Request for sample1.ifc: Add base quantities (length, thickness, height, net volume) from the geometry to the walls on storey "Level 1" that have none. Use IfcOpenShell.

First a look at what the model holds.

```python
import ifcopenshell
import ifcopenshell.util.element
import ifcopenshell.util.unit

model = ifcopenshell.open("sample1.ifc")
print(model.schema)
for unit_type in ("LENGTHUNIT", "AREAUNIT", "VOLUMEUNIT"):
    print(unit_type, ifcopenshell.util.unit.calculate_unit_scale(model, unit_type))
storey = next(s for s in model.by_type("IfcBuildingStorey") if s.Name == "Level 1")
walls = [e for e in ifcopenshell.util.element.get_decomposition(storey) if e.is_a("IfcWall")]
for e in sorted(walls, key=lambda e: e.id()):
    print(e.id(), e.is_a(), e.Name, list(ifcopenshell.util.element.get_psets(e, qtos_only=True)), sep=" | ")
```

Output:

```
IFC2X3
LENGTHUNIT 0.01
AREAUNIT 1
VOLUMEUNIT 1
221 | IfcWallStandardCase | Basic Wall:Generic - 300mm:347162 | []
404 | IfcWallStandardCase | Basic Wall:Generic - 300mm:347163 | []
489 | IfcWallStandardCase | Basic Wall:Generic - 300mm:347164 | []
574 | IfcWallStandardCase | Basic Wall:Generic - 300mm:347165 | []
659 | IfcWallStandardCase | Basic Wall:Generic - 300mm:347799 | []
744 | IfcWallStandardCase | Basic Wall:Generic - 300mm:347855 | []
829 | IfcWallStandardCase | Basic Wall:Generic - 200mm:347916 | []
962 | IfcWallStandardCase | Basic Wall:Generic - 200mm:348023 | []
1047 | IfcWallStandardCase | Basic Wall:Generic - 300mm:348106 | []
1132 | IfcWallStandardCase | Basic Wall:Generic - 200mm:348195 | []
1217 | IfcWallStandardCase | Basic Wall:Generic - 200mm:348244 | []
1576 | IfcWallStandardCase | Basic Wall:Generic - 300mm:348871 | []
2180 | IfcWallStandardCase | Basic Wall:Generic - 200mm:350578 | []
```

```python
import ifcopenshell
import ifcopenshell.api.pset
import ifcopenshell.geom
import ifcopenshell.util.element
import ifcopenshell.util.shape
import ifcopenshell.util.unit

model = ifcopenshell.open("sample1.ifc")
unit_scale = ifcopenshell.util.unit.calculate_unit_scale(model)
volume_scale = ifcopenshell.util.unit.calculate_unit_scale(model, "VOLUMEUNIT")
settings = ifcopenshell.geom.settings()

storey = next(s for s in model.by_type("IfcBuildingStorey") if s.Name == "Level 1")
walls = [e for e in ifcopenshell.util.element.get_decomposition(storey) if e.is_a("IfcWall")]

for e in sorted(walls, key=lambda e: e.id()):
    if ifcopenshell.util.element.get_psets(e, qtos_only=True, should_inherit=False):
        continue
    # Geometry comes back in metres, in the element's own axes.
    shape = ifcopenshell.geom.create_shape(settings, e)
    values = {
        "Length": ifcopenshell.util.shape.get_x(shape.geometry) / unit_scale,
        "Width": ifcopenshell.util.shape.get_y(shape.geometry) / unit_scale,
        "Height": ifcopenshell.util.shape.get_z(shape.geometry) / unit_scale,
        "NetVolume": ifcopenshell.util.shape.get_volume(shape.geometry) / volume_scale,
    }
    qto = ifcopenshell.api.pset.add_qto(model, product=e, name="BaseQuantities")
    ifcopenshell.api.pset.edit_qto(model, qto=qto, properties=values)
    print(e.id(), {k: round(v, 3) for k, v in values.items()})

model.write("sample1_edited.ifc")
```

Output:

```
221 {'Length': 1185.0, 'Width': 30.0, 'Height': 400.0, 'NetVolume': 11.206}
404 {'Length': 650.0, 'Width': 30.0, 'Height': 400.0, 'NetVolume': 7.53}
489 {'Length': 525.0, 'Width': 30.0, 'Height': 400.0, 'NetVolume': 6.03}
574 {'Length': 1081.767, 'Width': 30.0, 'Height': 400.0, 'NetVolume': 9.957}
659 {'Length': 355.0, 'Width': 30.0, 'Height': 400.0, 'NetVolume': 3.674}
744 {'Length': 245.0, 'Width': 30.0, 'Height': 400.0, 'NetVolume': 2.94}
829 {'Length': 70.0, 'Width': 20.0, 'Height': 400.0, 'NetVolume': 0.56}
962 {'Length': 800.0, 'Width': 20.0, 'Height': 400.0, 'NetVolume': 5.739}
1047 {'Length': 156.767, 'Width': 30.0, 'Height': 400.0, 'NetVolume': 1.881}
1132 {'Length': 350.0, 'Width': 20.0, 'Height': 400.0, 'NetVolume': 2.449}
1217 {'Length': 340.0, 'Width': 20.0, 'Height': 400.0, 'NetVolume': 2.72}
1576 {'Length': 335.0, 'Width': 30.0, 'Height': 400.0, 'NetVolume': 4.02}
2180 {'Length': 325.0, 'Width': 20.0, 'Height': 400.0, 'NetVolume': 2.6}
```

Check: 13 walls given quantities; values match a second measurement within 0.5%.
